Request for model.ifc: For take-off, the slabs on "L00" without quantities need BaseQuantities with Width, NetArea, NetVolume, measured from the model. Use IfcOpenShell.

First a look at what the model holds.

```python
import ifcopenshell
import ifcopenshell.util.element
import ifcopenshell.util.unit

model = ifcopenshell.open("model.ifc")
print(model.schema)
for unit_type in ("LENGTHUNIT", "AREAUNIT", "VOLUMEUNIT"):
    print(unit_type, ifcopenshell.util.unit.calculate_unit_scale(model, unit_type))
storey = next(s for s in model.by_type("IfcBuildingStorey") if s.Name == "L00")
slabs = [e for e in ifcopenshell.util.element.get_decomposition(storey) if e.is_a("IfcSlab")]
for e in sorted(slabs, key=lambda e: e.id()):
    print(e.id(), e.is_a(), e.Name, list(ifcopenshell.util.element.get_psets(e, qtos_only=True)), sep=" | ")
```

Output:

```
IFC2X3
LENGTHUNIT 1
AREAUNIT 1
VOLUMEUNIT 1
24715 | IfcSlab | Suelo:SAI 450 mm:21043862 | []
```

```python
import ifcopenshell
import ifcopenshell.api.pset
import ifcopenshell.geom
import ifcopenshell.util.element
import ifcopenshell.util.shape
import ifcopenshell.util.unit

model = ifcopenshell.open("model.ifc")
unit_scale = ifcopenshell.util.unit.calculate_unit_scale(model)
area_scale = ifcopenshell.util.unit.calculate_unit_scale(model, "AREAUNIT")
volume_scale = ifcopenshell.util.unit.calculate_unit_scale(model, "VOLUMEUNIT")
settings = ifcopenshell.geom.settings()

storey = next(s for s in model.by_type("IfcBuildingStorey") if s.Name == "L00")
slabs = [e for e in ifcopenshell.util.element.get_decomposition(storey) if e.is_a("IfcSlab")]

for e in sorted(slabs, key=lambda e: e.id()):
    if ifcopenshell.util.element.get_psets(e, qtos_only=True, should_inherit=False):
        continue
    # Geometry comes back in metres, in the element's own axes.
    shape = ifcopenshell.geom.create_shape(settings, e)
    values = {
        "Width": ifcopenshell.util.shape.get_z(shape.geometry) / unit_scale,
        "NetArea": ifcopenshell.util.shape.get_footprint_area(shape.geometry) / area_scale,
        "NetVolume": ifcopenshell.util.shape.get_volume(shape.geometry) / volume_scale,
    }
    qto = ifcopenshell.api.pset.add_qto(model, product=e, name="BaseQuantities")
    ifcopenshell.api.pset.edit_qto(model, qto=qto, properties=values)
    print(e.id(), {k: round(v, 3) for k, v in values.items()})

model.write("model_edited.ifc")
```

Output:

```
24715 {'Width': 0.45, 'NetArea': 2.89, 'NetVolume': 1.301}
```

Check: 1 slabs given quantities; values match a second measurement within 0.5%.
